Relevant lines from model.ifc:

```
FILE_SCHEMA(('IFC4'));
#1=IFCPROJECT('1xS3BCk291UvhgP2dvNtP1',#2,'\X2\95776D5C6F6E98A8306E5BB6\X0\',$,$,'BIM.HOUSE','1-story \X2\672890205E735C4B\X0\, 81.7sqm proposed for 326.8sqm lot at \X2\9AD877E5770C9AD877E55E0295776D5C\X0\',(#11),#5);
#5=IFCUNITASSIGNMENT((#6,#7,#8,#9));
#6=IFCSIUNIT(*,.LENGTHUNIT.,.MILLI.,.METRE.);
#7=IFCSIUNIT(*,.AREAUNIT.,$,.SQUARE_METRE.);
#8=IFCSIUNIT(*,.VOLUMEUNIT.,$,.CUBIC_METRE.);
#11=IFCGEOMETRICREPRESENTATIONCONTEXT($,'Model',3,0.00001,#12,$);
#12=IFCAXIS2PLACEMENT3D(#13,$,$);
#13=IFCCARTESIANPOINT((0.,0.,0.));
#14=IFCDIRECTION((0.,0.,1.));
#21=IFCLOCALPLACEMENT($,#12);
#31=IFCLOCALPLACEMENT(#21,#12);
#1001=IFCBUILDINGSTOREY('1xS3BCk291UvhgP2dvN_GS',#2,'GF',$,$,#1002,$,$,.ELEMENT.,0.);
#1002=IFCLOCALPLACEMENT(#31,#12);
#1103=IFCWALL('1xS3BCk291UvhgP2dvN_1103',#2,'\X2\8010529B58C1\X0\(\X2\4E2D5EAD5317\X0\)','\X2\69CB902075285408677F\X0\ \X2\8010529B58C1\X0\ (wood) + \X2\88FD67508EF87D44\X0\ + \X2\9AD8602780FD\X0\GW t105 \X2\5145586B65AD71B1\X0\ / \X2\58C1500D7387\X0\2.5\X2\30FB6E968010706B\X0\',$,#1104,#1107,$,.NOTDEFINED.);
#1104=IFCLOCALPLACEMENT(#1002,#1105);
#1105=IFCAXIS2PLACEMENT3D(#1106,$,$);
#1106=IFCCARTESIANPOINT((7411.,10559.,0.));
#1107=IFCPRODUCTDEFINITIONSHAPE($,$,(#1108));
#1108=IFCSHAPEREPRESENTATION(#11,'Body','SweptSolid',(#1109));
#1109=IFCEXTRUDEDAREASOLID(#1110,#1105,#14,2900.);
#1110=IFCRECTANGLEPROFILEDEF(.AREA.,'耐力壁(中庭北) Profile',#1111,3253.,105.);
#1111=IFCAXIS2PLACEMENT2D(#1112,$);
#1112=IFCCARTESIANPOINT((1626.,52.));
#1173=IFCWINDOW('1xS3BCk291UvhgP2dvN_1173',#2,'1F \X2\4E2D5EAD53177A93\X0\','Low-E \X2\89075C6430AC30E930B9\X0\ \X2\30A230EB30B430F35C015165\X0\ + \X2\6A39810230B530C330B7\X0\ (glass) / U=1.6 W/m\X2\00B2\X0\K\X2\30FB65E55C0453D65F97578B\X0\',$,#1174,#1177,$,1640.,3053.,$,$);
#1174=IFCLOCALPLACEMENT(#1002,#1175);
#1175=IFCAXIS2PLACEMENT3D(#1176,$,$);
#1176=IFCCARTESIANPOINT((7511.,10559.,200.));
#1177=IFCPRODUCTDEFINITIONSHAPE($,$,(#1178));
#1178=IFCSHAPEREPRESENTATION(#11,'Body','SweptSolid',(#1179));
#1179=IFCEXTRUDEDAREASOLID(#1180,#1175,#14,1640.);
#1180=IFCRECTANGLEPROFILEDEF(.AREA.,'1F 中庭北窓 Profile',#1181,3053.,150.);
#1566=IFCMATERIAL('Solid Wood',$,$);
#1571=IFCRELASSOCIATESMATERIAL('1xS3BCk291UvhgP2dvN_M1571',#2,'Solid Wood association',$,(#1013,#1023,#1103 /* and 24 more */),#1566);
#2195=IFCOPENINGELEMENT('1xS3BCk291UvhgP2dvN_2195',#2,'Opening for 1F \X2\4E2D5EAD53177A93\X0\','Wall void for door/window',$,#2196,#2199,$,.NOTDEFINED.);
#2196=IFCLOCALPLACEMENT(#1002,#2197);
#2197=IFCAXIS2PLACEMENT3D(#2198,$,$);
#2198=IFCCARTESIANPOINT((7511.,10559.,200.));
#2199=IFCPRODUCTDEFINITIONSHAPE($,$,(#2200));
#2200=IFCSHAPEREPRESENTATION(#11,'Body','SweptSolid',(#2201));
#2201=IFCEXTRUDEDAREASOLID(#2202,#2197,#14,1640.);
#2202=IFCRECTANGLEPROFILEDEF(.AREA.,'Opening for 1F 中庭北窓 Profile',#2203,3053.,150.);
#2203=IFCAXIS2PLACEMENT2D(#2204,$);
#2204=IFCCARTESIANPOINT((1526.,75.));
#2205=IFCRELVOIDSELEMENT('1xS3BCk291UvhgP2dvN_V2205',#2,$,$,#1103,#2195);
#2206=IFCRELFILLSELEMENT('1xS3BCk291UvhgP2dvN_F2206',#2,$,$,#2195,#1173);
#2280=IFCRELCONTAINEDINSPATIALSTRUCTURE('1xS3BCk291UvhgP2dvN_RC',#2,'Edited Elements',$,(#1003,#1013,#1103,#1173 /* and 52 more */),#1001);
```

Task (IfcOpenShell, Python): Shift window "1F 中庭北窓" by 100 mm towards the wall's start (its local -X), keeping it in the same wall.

```python
import ifcopenshell
import ifcopenshell.api.geometry
import ifcopenshell.util.placement

model = ifcopenshell.open("model.ifc")

window = model.by_id(1173)
opening = window.FillsVoids[0].RelatingOpeningElement
wall = opening.VoidsElements[0].RelatingBuildingElement

wall_matrix = ifcopenshell.util.placement.get_local_placement(wall.ObjectPlacement)
shift = wall_matrix[:3, 0] * -100.0
before = ifcopenshell.util.placement.get_local_placement(window.ObjectPlacement)[:3, 3].copy()

# The window is not placed relative to its opening, so move both.
for product in (opening, window):
    matrix = ifcopenshell.util.placement.get_local_placement(product.ObjectPlacement)
    matrix[:3, 3] += shift
    ifcopenshell.api.geometry.edit_object_placement(model, product=product, matrix=matrix, is_si=False)

after = ifcopenshell.util.placement.get_local_placement(window.ObjectPlacement)[:3, 3]
print("window moved by", (after - before).round(3) + 0.0)

model.write("model_edited.ifc")
```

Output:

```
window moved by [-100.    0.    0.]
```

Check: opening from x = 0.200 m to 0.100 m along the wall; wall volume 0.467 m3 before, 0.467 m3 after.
